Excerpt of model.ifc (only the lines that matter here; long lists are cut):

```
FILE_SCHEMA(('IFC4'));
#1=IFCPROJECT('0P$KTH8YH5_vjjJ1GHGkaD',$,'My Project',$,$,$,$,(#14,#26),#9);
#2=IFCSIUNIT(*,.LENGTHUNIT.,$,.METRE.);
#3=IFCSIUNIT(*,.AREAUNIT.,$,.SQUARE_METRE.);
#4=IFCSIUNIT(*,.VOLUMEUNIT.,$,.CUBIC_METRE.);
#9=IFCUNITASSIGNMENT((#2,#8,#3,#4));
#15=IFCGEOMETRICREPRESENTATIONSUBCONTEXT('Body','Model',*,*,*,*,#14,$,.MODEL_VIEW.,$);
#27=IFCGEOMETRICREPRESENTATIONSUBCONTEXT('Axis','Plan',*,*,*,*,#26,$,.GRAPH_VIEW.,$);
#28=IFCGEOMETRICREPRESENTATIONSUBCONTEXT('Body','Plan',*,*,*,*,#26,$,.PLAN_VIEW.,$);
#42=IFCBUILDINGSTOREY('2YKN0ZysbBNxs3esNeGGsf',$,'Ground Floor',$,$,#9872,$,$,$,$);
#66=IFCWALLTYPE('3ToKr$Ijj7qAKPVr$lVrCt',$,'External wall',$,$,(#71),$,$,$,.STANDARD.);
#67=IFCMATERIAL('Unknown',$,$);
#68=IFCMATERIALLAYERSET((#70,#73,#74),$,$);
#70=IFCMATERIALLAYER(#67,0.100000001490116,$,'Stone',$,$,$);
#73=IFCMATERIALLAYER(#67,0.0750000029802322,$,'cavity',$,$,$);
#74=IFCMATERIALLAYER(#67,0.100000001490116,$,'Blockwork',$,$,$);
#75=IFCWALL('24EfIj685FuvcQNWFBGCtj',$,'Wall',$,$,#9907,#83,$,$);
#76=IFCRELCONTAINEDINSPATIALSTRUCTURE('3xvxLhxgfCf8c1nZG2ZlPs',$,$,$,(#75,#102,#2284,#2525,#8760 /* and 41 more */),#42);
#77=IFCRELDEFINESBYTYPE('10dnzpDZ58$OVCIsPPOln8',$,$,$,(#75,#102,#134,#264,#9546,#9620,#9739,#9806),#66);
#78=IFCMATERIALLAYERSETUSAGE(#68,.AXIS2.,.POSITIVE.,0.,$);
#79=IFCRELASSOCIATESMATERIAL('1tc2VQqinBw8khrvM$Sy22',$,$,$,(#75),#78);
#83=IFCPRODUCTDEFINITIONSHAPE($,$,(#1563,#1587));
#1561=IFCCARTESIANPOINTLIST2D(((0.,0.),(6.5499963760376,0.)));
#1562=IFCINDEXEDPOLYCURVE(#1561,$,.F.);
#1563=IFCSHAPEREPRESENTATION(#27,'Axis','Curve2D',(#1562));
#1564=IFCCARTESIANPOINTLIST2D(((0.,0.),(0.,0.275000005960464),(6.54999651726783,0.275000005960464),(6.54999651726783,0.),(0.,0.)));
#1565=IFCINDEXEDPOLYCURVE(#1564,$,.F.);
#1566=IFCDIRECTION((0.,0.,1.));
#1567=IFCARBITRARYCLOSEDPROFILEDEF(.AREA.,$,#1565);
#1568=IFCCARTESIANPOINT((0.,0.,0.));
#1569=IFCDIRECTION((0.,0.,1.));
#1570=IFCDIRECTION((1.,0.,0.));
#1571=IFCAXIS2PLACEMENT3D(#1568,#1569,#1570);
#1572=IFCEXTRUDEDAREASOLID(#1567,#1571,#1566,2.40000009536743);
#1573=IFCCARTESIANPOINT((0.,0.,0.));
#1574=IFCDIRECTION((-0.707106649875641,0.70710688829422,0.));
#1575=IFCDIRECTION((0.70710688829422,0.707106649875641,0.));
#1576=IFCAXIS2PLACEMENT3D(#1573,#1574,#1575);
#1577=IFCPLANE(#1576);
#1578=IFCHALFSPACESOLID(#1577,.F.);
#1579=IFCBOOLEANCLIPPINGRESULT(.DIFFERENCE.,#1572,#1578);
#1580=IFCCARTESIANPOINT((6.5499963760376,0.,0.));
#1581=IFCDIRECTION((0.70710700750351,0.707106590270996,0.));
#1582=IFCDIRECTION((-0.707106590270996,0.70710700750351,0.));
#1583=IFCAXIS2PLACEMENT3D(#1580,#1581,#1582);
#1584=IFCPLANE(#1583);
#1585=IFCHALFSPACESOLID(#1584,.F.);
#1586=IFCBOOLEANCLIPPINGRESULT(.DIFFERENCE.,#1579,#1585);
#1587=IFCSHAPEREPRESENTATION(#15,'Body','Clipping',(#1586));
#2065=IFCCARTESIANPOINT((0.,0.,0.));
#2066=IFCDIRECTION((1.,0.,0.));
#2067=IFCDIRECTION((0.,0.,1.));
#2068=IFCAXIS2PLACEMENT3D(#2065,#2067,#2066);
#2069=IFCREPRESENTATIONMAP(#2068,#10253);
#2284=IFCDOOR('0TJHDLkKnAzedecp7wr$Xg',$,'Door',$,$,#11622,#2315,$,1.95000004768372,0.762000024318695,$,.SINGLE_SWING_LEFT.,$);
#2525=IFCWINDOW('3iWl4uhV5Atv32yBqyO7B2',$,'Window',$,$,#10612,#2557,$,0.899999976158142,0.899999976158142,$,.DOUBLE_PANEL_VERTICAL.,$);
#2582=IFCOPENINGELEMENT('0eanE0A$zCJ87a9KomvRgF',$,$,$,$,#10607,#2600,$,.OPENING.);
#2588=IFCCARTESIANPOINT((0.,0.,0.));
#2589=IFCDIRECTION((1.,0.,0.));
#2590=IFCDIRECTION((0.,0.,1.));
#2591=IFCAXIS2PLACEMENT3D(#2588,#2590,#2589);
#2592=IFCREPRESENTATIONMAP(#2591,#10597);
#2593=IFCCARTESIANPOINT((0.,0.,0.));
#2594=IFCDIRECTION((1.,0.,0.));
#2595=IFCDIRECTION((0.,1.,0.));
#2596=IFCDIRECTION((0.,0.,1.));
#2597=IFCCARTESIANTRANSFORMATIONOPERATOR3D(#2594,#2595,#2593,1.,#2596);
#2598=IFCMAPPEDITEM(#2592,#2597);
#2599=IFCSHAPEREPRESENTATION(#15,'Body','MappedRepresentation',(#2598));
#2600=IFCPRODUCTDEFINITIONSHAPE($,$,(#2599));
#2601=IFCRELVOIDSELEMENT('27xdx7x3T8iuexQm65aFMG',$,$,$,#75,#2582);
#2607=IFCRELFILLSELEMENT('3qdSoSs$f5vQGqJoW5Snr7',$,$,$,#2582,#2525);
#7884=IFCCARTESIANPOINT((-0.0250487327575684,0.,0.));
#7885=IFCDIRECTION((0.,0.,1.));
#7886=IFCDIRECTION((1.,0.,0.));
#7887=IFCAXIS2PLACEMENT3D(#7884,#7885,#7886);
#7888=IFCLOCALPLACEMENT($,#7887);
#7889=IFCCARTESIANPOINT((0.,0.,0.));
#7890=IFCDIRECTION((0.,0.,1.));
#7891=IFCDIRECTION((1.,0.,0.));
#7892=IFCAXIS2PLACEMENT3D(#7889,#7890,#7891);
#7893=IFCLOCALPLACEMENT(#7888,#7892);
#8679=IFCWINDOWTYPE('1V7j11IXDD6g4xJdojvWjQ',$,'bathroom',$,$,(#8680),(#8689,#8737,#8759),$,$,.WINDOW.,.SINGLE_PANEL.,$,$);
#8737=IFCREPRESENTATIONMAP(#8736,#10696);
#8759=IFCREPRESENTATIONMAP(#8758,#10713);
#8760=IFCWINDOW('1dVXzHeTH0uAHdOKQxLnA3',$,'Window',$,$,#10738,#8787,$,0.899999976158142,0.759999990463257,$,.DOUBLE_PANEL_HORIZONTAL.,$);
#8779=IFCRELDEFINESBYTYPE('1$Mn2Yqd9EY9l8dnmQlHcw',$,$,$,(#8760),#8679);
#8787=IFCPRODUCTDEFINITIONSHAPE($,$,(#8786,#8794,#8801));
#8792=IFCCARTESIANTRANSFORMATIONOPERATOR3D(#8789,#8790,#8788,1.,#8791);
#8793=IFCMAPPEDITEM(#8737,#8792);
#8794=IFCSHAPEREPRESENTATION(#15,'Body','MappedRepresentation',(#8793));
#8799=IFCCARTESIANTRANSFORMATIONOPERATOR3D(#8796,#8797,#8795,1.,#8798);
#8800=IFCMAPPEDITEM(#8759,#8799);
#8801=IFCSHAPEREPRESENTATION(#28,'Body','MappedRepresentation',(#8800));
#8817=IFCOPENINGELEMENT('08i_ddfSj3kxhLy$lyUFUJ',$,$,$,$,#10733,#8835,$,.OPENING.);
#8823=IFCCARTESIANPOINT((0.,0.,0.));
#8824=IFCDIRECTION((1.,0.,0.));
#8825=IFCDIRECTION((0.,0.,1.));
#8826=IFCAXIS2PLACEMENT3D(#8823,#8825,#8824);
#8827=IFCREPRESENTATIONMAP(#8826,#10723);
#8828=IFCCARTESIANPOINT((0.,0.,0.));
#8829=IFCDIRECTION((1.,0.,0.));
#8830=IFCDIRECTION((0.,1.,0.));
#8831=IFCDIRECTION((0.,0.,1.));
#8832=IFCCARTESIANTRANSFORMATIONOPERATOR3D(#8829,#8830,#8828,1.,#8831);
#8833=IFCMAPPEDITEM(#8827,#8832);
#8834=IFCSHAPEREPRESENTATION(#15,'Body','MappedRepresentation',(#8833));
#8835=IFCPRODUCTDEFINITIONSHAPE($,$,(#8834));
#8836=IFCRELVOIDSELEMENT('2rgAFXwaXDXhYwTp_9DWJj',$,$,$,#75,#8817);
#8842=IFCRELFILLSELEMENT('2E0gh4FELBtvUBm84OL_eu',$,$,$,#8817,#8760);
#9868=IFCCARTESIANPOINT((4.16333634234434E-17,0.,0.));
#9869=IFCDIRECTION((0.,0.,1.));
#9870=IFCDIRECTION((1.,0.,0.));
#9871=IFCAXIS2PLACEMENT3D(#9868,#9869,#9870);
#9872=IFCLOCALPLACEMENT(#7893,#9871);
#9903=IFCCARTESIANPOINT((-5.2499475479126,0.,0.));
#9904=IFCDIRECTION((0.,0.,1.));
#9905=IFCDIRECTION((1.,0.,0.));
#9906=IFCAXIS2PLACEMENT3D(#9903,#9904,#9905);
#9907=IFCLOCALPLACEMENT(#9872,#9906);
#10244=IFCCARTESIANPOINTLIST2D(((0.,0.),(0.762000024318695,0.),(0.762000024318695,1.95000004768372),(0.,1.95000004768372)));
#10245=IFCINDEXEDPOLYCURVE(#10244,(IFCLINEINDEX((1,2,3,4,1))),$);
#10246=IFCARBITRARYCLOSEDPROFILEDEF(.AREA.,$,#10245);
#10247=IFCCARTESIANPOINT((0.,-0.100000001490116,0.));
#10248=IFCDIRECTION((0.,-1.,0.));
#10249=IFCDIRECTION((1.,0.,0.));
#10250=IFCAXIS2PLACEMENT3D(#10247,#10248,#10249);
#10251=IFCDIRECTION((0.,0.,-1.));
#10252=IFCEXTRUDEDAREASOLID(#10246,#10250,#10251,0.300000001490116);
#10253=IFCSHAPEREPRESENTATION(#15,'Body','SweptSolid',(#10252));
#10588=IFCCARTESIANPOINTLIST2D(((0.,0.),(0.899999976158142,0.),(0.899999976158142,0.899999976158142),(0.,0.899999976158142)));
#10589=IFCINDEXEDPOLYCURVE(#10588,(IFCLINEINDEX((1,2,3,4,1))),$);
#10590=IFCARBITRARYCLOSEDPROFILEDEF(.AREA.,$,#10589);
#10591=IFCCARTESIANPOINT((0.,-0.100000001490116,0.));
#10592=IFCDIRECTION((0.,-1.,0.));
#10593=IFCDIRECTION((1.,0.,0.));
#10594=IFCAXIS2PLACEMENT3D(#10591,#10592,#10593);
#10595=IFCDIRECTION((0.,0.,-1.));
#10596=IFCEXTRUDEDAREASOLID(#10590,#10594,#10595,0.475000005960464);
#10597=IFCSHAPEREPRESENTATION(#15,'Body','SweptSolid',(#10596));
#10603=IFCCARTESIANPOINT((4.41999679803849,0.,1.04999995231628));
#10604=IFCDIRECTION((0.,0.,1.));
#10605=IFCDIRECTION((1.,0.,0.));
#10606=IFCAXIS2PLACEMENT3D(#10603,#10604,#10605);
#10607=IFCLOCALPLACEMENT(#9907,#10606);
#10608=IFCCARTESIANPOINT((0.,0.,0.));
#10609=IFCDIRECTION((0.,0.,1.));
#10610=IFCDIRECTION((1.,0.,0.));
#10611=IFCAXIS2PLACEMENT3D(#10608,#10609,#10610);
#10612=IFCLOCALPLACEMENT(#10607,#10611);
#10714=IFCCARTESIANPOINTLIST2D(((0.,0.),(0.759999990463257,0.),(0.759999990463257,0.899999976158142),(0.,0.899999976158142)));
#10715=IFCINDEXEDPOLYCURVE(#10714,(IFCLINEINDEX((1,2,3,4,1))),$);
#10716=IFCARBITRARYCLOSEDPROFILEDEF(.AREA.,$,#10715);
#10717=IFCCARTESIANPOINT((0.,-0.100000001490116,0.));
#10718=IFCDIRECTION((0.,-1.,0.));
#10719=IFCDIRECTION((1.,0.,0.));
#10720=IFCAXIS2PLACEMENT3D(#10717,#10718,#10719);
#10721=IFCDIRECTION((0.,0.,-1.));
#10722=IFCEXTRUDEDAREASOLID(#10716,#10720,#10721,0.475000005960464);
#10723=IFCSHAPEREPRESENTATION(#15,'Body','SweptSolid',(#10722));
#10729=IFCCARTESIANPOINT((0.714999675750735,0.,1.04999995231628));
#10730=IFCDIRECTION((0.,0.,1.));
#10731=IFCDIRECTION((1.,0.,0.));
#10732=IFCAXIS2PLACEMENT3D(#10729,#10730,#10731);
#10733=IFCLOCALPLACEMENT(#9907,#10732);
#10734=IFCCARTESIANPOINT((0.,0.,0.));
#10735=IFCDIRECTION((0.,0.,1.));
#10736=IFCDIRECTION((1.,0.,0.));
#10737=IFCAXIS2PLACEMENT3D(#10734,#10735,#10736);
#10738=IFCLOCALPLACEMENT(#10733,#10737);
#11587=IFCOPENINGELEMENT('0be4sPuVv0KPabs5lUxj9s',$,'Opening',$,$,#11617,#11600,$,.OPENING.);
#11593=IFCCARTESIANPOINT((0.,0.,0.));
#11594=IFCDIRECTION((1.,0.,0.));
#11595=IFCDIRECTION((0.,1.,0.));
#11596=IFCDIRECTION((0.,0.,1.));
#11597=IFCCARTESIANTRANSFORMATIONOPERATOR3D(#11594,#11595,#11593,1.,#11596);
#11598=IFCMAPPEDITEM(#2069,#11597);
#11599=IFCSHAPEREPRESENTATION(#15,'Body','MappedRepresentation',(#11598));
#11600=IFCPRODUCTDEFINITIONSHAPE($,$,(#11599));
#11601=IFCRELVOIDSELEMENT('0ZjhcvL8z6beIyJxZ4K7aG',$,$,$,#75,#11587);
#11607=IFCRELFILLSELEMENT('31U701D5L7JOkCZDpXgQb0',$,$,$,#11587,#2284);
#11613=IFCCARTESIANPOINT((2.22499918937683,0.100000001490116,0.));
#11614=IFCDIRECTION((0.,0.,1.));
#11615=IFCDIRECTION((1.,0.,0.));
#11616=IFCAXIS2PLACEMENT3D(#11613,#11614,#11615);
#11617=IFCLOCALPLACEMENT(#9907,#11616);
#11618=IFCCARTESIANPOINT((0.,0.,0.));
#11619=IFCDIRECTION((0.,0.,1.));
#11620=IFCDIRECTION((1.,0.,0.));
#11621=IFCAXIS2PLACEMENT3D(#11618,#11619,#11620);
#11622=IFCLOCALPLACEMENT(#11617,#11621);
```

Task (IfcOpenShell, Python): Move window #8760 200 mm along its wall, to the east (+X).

```python
import ifcopenshell
import ifcopenshell.api.geometry
import ifcopenshell.util.placement
import ifcopenshell.util.unit

model = ifcopenshell.open("model.ifc")
unit_scale = ifcopenshell.util.unit.calculate_unit_scale(model)

window = model.by_guid("1dVXzHeTH0uAHdOKQxLnA3")
opening = window.FillsVoids[0].RelatingOpeningElement
wall = opening.VoidsElements[0].RelatingBuildingElement

wall_matrix = ifcopenshell.util.placement.get_local_placement(wall.ObjectPlacement)
shift = wall_matrix[:3, 0] * 0.2 / unit_scale
before = ifcopenshell.util.placement.get_local_placement(window.ObjectPlacement)[:3, 3].copy()

# The window is placed relative to its opening, so it follows when the opening moves.
matrix = ifcopenshell.util.placement.get_local_placement(opening.ObjectPlacement)
matrix[:3, 3] += shift
ifcopenshell.api.geometry.edit_object_placement(
    model, product=opening, matrix=matrix, is_si=False, should_transform_children=True
)

after = ifcopenshell.util.placement.get_local_placement(window.ObjectPlacement)[:3, 3]
print("window moved by", (after - before).round(3) + 0.0)

model.write("model_updated.ifc")
```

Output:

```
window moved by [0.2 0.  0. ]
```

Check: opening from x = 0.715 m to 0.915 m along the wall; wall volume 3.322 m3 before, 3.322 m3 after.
